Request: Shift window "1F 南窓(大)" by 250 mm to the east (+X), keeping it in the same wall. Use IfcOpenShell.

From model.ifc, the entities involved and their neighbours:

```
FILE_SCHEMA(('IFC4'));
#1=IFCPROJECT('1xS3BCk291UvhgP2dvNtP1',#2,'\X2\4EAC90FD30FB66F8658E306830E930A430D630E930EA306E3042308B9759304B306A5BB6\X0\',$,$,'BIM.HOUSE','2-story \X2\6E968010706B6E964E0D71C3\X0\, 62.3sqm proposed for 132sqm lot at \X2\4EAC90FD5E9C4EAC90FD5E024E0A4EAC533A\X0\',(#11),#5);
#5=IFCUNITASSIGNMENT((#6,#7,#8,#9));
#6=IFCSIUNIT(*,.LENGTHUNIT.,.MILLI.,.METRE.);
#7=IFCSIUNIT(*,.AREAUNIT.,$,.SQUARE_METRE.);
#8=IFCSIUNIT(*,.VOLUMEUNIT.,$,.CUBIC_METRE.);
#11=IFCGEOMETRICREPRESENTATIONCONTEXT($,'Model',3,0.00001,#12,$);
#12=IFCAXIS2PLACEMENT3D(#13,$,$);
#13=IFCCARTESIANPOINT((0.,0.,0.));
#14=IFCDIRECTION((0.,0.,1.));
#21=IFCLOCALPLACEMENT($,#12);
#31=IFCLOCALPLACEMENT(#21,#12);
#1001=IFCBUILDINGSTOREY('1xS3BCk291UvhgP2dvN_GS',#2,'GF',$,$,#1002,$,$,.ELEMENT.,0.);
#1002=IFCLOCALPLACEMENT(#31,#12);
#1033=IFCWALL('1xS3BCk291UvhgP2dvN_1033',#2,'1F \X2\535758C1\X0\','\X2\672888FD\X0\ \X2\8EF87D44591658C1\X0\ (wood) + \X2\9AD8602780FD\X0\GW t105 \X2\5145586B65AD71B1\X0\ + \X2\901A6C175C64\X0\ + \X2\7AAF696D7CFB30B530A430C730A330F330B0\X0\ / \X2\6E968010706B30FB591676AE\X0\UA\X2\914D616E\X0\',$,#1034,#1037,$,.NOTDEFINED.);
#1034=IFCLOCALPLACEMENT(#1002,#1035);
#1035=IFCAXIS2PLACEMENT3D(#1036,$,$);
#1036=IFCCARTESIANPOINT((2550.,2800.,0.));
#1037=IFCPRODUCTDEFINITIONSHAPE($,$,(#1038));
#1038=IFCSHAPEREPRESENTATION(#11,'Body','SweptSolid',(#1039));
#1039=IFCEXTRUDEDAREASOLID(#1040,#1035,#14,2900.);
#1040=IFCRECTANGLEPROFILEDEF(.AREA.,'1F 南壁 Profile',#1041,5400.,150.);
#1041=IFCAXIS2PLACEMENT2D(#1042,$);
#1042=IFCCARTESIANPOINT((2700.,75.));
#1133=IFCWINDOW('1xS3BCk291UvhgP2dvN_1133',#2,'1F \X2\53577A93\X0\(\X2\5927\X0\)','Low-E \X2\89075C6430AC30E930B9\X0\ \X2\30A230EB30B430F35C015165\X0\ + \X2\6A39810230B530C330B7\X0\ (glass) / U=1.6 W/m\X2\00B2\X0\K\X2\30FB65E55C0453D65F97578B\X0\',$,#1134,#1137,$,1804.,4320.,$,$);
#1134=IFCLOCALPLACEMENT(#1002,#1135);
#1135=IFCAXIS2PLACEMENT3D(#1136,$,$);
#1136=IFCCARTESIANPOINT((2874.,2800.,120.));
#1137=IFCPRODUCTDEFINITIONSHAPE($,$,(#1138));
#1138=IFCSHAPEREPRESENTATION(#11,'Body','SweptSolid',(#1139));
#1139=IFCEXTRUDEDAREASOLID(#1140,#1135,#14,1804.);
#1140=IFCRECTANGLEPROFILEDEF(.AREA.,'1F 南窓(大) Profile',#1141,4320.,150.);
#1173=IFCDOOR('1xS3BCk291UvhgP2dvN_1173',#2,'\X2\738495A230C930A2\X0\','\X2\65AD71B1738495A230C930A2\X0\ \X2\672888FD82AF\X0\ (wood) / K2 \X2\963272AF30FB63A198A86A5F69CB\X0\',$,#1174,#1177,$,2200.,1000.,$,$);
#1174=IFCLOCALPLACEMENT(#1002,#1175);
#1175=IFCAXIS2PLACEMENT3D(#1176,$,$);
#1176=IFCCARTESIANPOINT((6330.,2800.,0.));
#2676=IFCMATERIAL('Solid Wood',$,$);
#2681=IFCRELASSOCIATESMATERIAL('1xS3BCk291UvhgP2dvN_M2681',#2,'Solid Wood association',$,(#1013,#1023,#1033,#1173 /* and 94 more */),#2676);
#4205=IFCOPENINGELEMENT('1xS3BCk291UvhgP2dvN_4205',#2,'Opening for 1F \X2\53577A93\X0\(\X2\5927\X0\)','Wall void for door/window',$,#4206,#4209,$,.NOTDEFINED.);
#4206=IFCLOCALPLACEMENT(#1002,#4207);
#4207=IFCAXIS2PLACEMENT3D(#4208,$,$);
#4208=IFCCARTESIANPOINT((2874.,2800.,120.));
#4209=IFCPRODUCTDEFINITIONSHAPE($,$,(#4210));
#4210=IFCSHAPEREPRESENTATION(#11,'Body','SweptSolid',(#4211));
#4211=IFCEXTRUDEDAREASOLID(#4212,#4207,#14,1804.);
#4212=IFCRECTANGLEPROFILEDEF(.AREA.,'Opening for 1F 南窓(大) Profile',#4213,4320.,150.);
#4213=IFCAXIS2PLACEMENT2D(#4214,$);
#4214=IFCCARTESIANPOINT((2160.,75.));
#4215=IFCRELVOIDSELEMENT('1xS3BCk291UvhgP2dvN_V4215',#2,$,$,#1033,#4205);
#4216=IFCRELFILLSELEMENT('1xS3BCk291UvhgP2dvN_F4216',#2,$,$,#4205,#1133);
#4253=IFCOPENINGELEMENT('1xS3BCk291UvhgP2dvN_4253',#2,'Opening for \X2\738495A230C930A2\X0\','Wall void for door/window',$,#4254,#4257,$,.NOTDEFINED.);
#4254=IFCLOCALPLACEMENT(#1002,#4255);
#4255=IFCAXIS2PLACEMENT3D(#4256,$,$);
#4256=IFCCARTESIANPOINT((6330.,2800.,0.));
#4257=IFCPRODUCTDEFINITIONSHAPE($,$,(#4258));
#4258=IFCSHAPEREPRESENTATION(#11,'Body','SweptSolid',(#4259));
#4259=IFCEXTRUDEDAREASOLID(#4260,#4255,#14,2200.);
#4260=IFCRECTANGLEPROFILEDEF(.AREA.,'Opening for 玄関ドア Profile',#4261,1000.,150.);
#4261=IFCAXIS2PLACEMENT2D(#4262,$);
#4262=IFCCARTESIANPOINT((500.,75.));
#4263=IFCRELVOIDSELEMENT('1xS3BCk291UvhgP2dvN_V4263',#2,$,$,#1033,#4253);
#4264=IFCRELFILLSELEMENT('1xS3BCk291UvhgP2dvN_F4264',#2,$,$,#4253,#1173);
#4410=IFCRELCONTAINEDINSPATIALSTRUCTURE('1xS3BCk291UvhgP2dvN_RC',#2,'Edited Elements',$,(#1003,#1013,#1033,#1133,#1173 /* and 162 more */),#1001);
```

```python
import ifcopenshell
import ifcopenshell.api.geometry
import ifcopenshell.util.placement

model = ifcopenshell.open("model.ifc")

window = model.by_guid("1xS3BCk291UvhgP2dvN_1133")
opening = window.FillsVoids[0].RelatingOpeningElement
wall = opening.VoidsElements[0].RelatingBuildingElement

wall_matrix = ifcopenshell.util.placement.get_local_placement(wall.ObjectPlacement)
shift = wall_matrix[:3, 0] * 250.0
before = ifcopenshell.util.placement.get_local_placement(window.ObjectPlacement)[:3, 3].copy()

# The window is not placed relative to its opening, so move both.
for product in (opening, window):
    matrix = ifcopenshell.util.placement.get_local_placement(product.ObjectPlacement)
    matrix[:3, 3] += shift
    ifcopenshell.api.geometry.edit_object_placement(model, product=product, matrix=matrix, is_si=False)

after = ifcopenshell.util.placement.get_local_placement(window.ObjectPlacement)[:3, 3]
print("window moved by", (after - before).round(3) + 0.0)

model.write("model_updated.ifc")
```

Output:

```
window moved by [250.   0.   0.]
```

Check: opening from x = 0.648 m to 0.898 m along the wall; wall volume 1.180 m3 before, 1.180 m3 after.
